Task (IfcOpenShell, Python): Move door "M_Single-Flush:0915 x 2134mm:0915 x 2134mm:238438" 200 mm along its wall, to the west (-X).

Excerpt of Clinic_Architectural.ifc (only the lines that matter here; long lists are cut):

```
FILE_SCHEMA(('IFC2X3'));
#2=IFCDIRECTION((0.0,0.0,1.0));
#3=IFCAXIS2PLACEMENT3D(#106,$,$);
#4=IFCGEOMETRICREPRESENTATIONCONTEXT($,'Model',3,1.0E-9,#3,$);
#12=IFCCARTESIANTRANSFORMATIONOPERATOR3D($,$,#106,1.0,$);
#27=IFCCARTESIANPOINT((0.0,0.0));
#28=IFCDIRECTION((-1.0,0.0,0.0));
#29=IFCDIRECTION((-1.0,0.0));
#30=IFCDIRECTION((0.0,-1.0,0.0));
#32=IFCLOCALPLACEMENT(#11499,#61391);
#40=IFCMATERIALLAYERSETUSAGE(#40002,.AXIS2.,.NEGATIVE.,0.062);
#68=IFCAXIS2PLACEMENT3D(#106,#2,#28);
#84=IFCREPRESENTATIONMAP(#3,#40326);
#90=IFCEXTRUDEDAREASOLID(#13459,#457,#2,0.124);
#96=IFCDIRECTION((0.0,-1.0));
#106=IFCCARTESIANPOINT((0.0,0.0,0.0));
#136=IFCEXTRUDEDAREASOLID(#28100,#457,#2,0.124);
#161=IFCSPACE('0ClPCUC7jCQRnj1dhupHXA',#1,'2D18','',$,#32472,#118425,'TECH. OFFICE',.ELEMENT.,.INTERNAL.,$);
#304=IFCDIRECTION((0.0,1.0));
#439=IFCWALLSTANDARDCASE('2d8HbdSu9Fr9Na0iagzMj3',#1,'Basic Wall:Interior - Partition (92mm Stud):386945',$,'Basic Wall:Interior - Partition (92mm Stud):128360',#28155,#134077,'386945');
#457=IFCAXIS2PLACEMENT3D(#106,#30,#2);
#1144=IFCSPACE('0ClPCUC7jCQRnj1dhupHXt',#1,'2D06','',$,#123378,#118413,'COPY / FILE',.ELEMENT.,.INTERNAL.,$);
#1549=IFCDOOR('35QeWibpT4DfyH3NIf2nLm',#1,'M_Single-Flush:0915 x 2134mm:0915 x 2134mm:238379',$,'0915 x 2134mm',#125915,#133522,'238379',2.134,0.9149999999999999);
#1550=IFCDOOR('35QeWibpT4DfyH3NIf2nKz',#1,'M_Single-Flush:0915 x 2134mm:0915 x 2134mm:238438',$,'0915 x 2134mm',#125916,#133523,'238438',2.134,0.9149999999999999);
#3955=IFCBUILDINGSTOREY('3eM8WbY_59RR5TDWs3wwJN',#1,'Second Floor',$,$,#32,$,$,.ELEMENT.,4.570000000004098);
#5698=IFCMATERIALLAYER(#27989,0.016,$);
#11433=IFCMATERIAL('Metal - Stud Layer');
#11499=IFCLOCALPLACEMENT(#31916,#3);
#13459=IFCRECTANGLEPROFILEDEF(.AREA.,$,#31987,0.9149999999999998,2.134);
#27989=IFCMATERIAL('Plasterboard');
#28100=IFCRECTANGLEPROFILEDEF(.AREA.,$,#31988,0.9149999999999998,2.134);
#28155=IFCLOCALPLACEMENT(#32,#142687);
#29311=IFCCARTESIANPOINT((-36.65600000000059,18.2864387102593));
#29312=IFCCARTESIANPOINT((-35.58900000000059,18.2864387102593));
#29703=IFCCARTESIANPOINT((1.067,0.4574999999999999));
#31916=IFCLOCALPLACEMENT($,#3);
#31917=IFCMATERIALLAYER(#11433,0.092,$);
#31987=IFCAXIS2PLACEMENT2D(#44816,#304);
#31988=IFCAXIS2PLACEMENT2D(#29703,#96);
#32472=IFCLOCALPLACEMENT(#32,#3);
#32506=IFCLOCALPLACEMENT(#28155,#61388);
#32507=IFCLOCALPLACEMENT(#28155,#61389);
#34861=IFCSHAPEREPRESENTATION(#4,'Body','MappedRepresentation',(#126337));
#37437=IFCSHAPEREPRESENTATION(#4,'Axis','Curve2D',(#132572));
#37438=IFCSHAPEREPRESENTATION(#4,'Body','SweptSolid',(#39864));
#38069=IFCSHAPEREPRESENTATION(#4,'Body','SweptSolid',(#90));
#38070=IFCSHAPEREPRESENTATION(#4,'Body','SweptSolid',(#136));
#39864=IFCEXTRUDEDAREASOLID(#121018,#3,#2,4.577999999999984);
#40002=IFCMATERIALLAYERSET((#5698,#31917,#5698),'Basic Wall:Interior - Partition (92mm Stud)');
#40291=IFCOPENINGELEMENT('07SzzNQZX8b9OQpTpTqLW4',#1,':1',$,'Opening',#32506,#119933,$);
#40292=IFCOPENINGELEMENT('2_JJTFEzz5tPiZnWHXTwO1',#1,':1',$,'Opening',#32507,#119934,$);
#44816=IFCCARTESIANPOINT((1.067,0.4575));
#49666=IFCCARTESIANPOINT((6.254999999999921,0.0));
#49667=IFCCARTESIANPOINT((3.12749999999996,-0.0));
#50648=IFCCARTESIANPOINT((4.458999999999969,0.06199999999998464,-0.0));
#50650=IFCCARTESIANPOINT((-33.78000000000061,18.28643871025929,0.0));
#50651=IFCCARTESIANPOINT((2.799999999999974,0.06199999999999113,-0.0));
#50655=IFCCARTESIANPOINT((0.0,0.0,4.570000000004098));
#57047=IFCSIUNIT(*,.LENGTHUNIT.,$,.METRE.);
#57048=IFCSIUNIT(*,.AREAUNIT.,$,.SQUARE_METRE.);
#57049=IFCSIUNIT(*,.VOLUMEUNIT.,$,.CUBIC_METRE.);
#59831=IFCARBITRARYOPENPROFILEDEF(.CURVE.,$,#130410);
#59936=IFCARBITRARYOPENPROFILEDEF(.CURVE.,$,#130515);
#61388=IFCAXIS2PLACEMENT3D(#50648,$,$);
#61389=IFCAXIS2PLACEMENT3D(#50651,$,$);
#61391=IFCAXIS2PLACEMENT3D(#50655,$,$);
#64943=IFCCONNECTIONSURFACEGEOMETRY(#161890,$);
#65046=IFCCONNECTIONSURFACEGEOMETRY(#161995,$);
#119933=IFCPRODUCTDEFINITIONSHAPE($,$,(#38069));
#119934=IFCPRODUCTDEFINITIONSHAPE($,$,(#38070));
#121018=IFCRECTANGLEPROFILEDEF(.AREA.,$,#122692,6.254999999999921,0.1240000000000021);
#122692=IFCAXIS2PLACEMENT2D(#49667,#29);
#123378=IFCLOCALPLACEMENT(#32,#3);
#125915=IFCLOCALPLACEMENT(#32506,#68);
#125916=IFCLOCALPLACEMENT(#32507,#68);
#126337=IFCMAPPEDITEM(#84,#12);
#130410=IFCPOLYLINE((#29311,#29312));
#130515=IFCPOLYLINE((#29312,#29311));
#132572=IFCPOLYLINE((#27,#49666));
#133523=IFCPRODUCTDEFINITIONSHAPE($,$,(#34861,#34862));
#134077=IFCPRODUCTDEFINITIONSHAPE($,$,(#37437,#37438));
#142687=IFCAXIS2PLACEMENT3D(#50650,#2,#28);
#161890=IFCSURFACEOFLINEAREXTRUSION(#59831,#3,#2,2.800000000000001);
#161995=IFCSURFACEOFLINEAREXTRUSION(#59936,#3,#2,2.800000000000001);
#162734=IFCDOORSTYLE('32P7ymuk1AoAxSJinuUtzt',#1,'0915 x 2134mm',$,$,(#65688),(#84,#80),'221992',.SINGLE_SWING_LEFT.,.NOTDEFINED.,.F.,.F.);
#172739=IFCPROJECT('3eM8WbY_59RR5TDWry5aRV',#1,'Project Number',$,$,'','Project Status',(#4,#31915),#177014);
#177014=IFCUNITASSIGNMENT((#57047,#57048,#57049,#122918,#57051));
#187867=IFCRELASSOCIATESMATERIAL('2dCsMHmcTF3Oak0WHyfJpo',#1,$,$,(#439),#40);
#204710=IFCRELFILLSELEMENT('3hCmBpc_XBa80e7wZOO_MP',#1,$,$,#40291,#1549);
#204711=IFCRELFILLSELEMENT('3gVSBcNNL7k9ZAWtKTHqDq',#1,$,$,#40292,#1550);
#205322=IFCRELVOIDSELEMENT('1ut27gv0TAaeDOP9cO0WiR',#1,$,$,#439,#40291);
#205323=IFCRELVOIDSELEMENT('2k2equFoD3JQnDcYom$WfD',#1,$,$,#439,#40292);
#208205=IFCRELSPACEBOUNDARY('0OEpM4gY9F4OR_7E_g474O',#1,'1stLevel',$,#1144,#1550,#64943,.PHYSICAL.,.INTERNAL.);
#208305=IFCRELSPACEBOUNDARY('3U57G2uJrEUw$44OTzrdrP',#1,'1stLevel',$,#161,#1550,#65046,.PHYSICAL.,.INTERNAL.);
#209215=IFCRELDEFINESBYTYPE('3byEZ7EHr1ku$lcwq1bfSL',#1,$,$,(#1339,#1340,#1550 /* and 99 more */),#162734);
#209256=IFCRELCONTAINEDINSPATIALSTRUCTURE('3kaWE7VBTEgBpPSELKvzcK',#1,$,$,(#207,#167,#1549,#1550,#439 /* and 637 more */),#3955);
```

```python
import numpy as np
import ifcopenshell
import ifcopenshell.api.geometry
import ifcopenshell.util.placement
import ifcopenshell.util.unit

model = ifcopenshell.open("Clinic_Architectural.ifc")
unit_scale = ifcopenshell.util.unit.calculate_unit_scale(model)

door = model.by_id(1550)
opening = door.FillsVoids[0].RelatingOpeningElement
wall = opening.VoidsElements[0].RelatingBuildingElement

wall_matrix = ifcopenshell.util.placement.get_local_placement(wall.ObjectPlacement)
shift = wall_matrix[:3, 0] * 0.2 / unit_scale
before = ifcopenshell.util.placement.get_local_placement(door.ObjectPlacement)[:3, 3].copy()

# The door is placed relative to its opening, so it follows when the opening moves.
matrix = ifcopenshell.util.placement.get_local_placement(opening.ObjectPlacement)
matrix[:3, 3] += shift
ifcopenshell.api.geometry.edit_object_placement(
    model, product=opening, matrix=matrix, is_si=False, should_transform_children=True
)

# Space boundary surfaces are stored in each space's coordinates; move them too.
for rel in door.ProvidesBoundaries:
    if not rel.ConnectionGeometry:
        continue
    surface = rel.ConnectionGeometry.SurfaceOnRelatingElement
    space_matrix = ifcopenshell.util.placement.get_local_placement(rel.RelatingSpace.ObjectPlacement)
    point = np.array(surface.Position.Location.Coordinates) + space_matrix[:3, :3].T @ shift
    surface.Position = model.createIfcAxis2Placement3D(
        model.createIfcCartesianPoint(point.tolist()), surface.Position.Axis, surface.Position.RefDirection
    )

after = ifcopenshell.util.placement.get_local_placement(door.ObjectPlacement)[:3, 3]
print("door moved by", (after - before).round(3) + 0.0)

model.write("Clinic_Architectural_edited.ifc")
```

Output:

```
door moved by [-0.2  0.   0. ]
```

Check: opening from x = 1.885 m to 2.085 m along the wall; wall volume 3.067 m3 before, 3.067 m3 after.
